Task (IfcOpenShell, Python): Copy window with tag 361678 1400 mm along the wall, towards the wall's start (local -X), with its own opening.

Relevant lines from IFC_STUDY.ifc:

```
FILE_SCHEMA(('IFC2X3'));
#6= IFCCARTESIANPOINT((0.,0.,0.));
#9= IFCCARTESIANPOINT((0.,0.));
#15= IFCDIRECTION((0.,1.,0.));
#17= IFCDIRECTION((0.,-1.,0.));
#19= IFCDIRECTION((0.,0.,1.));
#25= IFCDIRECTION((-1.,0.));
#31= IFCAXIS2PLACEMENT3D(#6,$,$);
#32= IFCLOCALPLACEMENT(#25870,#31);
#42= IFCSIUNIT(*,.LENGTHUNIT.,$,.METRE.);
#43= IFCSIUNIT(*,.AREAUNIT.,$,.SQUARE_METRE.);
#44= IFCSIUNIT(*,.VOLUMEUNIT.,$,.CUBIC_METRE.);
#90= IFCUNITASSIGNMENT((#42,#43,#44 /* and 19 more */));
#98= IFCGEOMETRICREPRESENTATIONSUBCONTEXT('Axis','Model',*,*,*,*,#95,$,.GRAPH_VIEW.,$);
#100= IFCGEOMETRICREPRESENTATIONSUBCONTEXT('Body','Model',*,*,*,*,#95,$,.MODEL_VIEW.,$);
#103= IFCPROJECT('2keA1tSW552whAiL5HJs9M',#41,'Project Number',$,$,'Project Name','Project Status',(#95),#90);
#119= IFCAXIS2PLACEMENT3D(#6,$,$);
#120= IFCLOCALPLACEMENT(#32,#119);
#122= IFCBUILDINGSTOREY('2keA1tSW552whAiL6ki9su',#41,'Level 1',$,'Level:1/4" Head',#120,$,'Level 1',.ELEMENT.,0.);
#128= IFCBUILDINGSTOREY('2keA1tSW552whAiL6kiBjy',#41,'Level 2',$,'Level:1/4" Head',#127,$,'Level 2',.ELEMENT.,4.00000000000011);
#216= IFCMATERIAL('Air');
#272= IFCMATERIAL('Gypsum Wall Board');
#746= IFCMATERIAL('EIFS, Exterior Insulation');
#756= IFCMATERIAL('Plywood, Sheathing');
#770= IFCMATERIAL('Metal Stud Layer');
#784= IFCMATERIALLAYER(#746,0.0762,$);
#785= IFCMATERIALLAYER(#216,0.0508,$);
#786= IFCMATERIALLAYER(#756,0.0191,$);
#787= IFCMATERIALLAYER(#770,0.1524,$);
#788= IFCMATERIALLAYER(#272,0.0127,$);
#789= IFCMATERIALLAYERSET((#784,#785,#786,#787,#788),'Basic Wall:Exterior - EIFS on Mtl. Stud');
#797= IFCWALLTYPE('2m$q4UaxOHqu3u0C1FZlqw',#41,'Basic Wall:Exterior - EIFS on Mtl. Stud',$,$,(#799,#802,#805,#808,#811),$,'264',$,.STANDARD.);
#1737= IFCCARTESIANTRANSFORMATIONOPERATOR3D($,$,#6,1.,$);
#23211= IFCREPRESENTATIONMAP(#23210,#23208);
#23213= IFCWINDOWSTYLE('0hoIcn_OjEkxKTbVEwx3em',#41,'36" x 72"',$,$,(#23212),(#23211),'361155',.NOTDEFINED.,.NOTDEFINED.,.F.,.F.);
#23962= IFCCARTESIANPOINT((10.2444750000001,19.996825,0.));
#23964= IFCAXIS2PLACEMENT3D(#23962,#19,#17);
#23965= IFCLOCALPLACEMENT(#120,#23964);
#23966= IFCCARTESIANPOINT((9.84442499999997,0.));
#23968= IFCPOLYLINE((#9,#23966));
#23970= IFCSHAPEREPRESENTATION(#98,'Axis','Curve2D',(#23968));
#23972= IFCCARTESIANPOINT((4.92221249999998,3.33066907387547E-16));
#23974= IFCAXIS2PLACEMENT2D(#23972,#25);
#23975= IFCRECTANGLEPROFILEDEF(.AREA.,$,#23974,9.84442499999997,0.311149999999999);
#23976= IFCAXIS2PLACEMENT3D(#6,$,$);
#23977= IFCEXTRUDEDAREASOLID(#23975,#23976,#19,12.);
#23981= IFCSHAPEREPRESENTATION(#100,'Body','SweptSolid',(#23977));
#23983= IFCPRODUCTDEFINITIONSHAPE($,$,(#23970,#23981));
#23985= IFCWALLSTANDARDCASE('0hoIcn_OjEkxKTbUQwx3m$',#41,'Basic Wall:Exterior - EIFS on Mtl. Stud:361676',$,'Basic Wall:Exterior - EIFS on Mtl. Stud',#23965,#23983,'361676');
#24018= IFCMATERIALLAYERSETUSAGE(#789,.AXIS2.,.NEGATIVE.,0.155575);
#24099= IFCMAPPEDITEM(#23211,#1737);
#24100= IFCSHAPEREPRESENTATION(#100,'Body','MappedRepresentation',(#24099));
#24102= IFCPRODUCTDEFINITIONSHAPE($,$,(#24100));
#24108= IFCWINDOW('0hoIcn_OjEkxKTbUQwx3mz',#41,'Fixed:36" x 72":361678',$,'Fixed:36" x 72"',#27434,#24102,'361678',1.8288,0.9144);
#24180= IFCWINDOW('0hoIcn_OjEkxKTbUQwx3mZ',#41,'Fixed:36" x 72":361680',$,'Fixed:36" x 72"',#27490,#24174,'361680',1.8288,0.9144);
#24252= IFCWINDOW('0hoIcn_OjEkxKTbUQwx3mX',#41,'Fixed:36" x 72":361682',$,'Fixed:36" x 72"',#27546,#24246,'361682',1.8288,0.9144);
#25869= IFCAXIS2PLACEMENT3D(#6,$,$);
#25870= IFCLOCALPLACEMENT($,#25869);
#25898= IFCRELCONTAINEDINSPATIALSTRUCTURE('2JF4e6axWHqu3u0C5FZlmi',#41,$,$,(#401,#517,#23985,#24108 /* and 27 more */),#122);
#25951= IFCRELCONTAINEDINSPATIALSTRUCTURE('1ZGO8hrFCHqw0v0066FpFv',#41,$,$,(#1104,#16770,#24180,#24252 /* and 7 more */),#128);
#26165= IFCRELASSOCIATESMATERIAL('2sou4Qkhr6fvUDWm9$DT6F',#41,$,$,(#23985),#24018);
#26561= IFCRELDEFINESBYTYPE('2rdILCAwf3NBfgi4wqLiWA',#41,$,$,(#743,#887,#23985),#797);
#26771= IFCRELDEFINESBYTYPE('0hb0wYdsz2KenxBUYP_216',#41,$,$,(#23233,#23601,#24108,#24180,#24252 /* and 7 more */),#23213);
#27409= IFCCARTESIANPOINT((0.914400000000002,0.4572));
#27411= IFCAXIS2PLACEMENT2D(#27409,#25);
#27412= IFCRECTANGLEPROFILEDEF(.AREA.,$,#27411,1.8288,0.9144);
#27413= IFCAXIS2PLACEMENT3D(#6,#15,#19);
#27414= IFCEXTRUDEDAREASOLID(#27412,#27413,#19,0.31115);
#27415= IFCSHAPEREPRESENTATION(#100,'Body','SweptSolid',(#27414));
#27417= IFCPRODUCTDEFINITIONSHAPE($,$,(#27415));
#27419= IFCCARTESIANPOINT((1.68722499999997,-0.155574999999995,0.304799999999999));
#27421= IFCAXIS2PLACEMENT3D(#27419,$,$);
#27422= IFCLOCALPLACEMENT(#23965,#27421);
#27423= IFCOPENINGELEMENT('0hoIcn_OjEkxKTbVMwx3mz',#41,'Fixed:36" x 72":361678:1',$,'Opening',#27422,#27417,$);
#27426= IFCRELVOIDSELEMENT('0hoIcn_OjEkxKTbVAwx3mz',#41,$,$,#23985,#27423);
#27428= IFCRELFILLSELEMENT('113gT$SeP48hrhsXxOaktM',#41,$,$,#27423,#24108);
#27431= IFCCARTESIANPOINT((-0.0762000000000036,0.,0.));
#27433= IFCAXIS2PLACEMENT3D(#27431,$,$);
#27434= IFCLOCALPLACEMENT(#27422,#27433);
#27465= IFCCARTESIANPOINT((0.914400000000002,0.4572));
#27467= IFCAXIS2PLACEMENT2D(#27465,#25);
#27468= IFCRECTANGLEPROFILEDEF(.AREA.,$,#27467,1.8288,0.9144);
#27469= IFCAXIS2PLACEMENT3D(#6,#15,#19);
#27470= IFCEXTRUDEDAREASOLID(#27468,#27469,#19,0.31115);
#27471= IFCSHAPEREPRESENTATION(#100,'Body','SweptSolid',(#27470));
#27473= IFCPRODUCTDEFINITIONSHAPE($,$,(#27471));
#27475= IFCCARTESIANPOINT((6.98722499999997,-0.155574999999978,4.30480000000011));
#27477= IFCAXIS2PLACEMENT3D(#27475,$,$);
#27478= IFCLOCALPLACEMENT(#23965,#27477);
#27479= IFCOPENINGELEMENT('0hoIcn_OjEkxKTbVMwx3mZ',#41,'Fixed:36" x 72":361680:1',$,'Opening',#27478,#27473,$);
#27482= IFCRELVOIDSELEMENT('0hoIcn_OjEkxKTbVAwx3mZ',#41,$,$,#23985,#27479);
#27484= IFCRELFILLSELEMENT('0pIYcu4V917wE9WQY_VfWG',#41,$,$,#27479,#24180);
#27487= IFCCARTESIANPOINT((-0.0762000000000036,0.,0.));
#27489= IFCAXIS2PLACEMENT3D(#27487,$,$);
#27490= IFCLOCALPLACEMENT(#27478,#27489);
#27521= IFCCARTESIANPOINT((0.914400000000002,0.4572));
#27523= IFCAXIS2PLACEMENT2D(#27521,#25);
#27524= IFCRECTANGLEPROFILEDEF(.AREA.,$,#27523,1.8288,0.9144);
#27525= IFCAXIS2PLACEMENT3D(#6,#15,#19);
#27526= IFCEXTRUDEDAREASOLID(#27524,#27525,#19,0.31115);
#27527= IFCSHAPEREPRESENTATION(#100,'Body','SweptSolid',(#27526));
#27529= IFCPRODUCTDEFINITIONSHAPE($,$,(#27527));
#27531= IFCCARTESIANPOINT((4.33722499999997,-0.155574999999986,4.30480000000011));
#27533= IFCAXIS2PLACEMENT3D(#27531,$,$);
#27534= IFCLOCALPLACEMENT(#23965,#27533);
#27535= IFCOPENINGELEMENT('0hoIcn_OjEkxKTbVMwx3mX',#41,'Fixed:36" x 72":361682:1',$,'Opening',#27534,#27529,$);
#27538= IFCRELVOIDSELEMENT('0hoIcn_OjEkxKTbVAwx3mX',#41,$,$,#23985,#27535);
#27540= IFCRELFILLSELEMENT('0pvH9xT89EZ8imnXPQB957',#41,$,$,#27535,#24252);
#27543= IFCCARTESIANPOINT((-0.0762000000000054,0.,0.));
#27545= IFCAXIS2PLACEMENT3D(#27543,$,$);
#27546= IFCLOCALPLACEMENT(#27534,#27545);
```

```python
import ifcopenshell
import ifcopenshell.api.feature
import ifcopenshell.api.geometry
import ifcopenshell.api.root
import ifcopenshell.geom
import ifcopenshell.util.element
import ifcopenshell.util.placement
import ifcopenshell.util.shape
import ifcopenshell.util.unit

model = ifcopenshell.open("IFC_STUDY.ifc")
unit_scale = ifcopenshell.util.unit.calculate_unit_scale(model)
settings = ifcopenshell.geom.settings()


def volume(element):
    """Net volume in cubic metres, openings subtracted."""
    shape = ifcopenshell.geom.create_shape(settings, element)
    return ifcopenshell.util.shape.get_volume(shape.geometry)


def reuse_history(source, copy):
    """copy_class also copies each property set's owner history, people and application; keep the originals."""
    for rel in copy.IsDefinedBy:
        if rel.is_a("IfcRelDefinesByProperties") and (history := rel.RelatingPropertyDefinition.OwnerHistory):
            rel.RelatingPropertyDefinition.OwnerHistory = source.OwnerHistory
            ifcopenshell.util.element.remove_deep2(model, history)


window = model.by_guid("0hoIcn_OjEkxKTbUQwx3mz")
opening = window.FillsVoids[0].RelatingOpeningElement
wall = opening.VoidsElements[0].RelatingBuildingElement
before = volume(wall)
shift = ifcopenshell.util.placement.get_local_placement(wall.ObjectPlacement)[:3, 0] * -1.4 / unit_scale

# copy_class copies the void relationship, type, container and properties, but no geometry.
new_opening = ifcopenshell.api.root.copy_class(model, product=opening)
new_opening.Representation = ifcopenshell.util.element.copy_deep(
    model, opening.Representation, exclude=["IfcGeometricRepresentationContext", "IfcRepresentationMap"]
)
new_opening.Name = 'Fixed:36" x 72"'
new_window = ifcopenshell.api.root.copy_class(model, product=window)
new_window.Representation = ifcopenshell.util.element.copy_deep(
    model, window.Representation, exclude=["IfcGeometricRepresentationContext", "IfcRepresentationMap"]
)
new_window.Name = 'Fixed:36" x 72"'
new_window.Tag = None
reuse_history(window, new_window)
fills = ifcopenshell.api.feature.add_filling(model, opening=new_opening, element=new_window)
fills.OwnerHistory = new_window.OwnerHistory  # required in IFC2X3

for old, new in ((opening, new_opening), (window, new_window)):
    matrix = ifcopenshell.util.placement.get_local_placement(old.ObjectPlacement)
    matrix[:3, 3] += shift
    ifcopenshell.api.geometry.edit_object_placement(model, product=new, matrix=matrix, is_si=False)

after = volume(wall)

print(f"wall volume {before:.3f} -> {after:.3f} m3")

model.write("IFC_STUDY_v2.ifc")
```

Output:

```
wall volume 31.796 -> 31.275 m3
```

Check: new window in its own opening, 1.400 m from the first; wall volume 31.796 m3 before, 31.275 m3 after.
